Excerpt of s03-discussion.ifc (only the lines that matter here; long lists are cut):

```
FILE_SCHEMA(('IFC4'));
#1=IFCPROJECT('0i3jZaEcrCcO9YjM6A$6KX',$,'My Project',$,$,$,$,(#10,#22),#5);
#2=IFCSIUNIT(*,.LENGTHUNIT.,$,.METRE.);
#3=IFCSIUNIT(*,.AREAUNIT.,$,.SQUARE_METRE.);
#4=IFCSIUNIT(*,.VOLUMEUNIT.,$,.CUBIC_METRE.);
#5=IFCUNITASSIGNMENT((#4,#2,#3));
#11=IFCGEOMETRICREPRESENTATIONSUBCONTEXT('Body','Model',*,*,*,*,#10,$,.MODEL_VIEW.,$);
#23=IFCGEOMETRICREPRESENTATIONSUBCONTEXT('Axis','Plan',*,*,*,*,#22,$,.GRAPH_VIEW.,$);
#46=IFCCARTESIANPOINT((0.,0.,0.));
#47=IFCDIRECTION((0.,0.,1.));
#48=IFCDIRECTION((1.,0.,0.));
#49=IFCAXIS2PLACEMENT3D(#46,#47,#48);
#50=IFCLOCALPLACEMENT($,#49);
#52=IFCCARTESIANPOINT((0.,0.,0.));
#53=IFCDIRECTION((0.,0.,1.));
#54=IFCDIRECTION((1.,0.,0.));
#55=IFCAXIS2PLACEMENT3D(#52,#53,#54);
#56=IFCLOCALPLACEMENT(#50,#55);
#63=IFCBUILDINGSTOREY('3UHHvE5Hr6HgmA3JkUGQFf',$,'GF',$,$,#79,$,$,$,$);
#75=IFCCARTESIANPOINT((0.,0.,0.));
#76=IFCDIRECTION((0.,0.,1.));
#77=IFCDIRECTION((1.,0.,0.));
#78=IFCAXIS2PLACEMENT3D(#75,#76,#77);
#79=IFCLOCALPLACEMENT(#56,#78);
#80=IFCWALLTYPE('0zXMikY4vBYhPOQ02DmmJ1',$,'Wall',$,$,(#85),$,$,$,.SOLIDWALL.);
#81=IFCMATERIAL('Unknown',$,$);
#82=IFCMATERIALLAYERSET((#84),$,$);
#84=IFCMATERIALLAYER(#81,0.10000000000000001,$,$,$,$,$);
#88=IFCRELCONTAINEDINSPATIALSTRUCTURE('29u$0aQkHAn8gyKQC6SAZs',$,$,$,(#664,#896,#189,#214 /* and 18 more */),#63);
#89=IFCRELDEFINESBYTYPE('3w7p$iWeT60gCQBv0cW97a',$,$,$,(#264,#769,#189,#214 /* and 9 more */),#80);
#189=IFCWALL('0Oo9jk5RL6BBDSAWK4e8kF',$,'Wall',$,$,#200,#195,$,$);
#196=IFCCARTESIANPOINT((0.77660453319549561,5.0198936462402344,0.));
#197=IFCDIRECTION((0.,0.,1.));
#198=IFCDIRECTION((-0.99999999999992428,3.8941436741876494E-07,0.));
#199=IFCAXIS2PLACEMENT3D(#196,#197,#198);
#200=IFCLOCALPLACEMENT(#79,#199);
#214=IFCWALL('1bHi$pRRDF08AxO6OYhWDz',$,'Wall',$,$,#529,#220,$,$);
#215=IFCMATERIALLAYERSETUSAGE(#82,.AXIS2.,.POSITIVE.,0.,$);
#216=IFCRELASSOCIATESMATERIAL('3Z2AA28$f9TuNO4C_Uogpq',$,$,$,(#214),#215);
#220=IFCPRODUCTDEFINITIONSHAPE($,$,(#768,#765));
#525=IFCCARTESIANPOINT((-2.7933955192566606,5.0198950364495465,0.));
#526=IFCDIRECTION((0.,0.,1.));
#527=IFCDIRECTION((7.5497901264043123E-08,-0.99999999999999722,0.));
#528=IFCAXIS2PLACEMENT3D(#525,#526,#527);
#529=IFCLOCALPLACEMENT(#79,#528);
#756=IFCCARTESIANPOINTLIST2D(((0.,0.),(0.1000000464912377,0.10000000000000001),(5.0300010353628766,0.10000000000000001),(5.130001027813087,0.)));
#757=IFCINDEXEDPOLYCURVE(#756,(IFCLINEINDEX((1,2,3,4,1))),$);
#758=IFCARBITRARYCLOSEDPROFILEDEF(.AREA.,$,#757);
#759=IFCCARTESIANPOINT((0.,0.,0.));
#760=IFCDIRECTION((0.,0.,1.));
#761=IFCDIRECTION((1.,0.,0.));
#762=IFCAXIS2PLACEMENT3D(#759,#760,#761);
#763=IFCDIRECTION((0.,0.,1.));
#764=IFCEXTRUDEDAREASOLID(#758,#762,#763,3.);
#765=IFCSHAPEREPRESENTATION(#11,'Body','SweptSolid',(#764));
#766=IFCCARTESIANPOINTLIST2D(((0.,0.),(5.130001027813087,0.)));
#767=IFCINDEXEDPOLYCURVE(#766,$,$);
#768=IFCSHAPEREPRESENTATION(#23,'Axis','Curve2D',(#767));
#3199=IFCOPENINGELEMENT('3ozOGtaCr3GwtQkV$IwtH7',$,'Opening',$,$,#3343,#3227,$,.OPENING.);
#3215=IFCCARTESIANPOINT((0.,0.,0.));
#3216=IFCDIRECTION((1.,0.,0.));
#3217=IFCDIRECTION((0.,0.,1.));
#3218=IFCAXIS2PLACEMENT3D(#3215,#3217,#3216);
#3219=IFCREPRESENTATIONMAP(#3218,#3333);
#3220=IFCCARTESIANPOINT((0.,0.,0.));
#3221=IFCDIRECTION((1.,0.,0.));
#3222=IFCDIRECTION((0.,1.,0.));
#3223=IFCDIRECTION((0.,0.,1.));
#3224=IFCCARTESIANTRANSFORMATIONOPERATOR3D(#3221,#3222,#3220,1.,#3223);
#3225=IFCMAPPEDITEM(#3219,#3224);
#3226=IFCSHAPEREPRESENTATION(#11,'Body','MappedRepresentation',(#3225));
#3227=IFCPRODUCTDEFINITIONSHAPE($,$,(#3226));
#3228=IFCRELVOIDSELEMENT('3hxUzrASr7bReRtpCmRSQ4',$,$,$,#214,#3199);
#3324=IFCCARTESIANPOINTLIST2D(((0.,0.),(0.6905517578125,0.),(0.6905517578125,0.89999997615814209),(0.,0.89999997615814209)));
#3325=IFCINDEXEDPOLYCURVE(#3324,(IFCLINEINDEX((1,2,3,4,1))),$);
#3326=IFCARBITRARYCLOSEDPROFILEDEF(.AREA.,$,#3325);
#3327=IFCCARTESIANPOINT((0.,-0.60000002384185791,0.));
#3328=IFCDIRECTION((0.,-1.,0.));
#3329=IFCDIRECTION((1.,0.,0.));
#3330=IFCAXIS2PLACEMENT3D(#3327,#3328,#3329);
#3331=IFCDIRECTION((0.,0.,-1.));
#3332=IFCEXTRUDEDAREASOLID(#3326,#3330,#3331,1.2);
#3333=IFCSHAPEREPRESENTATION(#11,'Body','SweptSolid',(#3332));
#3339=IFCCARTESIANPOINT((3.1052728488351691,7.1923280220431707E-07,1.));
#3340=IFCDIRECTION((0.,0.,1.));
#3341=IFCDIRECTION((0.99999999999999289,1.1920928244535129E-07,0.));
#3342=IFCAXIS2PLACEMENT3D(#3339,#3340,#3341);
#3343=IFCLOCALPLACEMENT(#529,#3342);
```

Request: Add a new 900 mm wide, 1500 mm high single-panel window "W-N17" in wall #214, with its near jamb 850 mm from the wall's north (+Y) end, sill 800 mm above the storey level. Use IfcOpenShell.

```python
import numpy as np
import ifcopenshell
import ifcopenshell.api.feature
import ifcopenshell.api.geometry
import ifcopenshell.api.root
import ifcopenshell.api.spatial
import ifcopenshell.geom
import ifcopenshell.util.element
import ifcopenshell.util.placement
import ifcopenshell.util.representation
import ifcopenshell.util.shape
import ifcopenshell.util.unit

model = ifcopenshell.open("s03-discussion.ifc")
unit_scale = ifcopenshell.util.unit.calculate_unit_scale(model)
settings = ifcopenshell.geom.settings()


def volume(element):
    """Net volume in cubic metres, openings subtracted."""
    shape = ifcopenshell.geom.create_shape(settings, element)
    return ifcopenshell.util.shape.get_volume(shape.geometry)


wall = model.by_id(214)
storey = ifcopenshell.util.element.get_container(wall, ifc_class="IfcBuildingStorey")
context = ifcopenshell.util.representation.get_context(model, "Model", "Body", "MODEL_VIEW")
before = volume(wall)

width, height, from_end, sill = 0.9, 1.5, 0.85, 0.8  # metres

# The wall runs along its own X axis, and the end named is its -X end.
wall_shape = ifcopenshell.geom.create_shape(settings, wall)
x, y, z = ifcopenshell.util.shape.get_vertices(wall_shape.geometry).T
start = x.min() + from_end
face, thickness = float(y.min()), float(y.max() - y.min())
wall_matrix = ifcopenshell.util.placement.get_local_placement(wall.ObjectPlacement)
level = ifcopenshell.util.placement.get_local_placement(storey.ObjectPlacement)[2, 3]


def in_wall(x, y):
    """Placement at x, y metres in the wall's axes, at sill height."""
    matrix = wall_matrix.copy()
    matrix[:, 3] = wall_matrix @ np.array([x / unit_scale, y / unit_scale, 0.0, 1.0])
    matrix[2, 3] = level + sill / unit_scale
    return matrix


# Opening: a box that overshoots both wall faces by 50 mm.
opening = ifcopenshell.api.root.create_entity(model, ifc_class="IfcOpeningElement", predefined_type="OPENING")
box = ifcopenshell.api.geometry.add_wall_representation(
    model, context=context, length=width, height=height, thickness=thickness + 0.1
)
ifcopenshell.api.geometry.assign_representation(model, product=opening, representation=box)
ifcopenshell.api.geometry.edit_object_placement(model, product=opening, matrix=in_wall(start, face - 0.05), is_si=False)
ifcopenshell.api.feature.add_feature(model, feature=opening, element=wall)

window = ifcopenshell.api.root.create_entity(model, ifc_class="IfcWindow", name="W-N17", predefined_type="WINDOW")
window.OverallWidth, window.OverallHeight = width / unit_scale, height / unit_scale
window.PartitioningType = "SINGLE_PANEL"
body = ifcopenshell.api.geometry.add_window_representation(
    model,
    context=context,
    overall_width=window.OverallWidth,
    overall_height=window.OverallHeight,
    partition_type="SINGLE_PANEL",
)
ifcopenshell.api.geometry.assign_representation(model, product=window, representation=body)
ifcopenshell.api.spatial.assign_container(model, products=[window], relating_structure=storey)
ifcopenshell.api.feature.add_filling(model, opening=opening, element=window)

# Centre the window in the wall's thickness.
ifcopenshell.api.geometry.edit_object_placement(model, product=window, matrix=in_wall(start, face), is_si=False)
window_shape = ifcopenshell.geom.create_shape(settings, window)
depth = ifcopenshell.util.shape.get_vertices(window_shape.geometry)[:, 1]
offset = face + thickness / 2 - (depth.min() + depth.max()) / 2
ifcopenshell.api.geometry.edit_object_placement(model, product=window, matrix=in_wall(start, offset), is_si=False)

after = volume(wall)

print(f"wall volume {before:.3f} -> {after:.3f} m3")

model.write("s03-discussion_edited.ifc")
```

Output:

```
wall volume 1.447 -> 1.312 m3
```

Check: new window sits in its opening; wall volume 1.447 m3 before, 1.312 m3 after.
